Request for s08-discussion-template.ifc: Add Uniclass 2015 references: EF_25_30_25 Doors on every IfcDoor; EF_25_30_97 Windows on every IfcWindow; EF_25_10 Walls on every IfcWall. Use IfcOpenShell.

First a look at what the model holds.

```python
import ifcopenshell

model = ifcopenshell.open("s08-discussion-template.ifc")
print(model.schema)
print("classifications:", [c.Name for c in model.by_type("IfcClassification")])
for ifc_class in ("IfcDoor", "IfcRoof", "IfcStair", "IfcWall", "IfcWindow"):
    print(ifc_class, len(model.by_type(ifc_class)))
```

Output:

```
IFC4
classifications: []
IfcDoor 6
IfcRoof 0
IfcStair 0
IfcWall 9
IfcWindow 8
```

```python
import ifcopenshell
import ifcopenshell.api.classification

model = ifcopenshell.open("s08-discussion-template.ifc")

system = ifcopenshell.api.classification.add_classification(model, classification="Uniclass 2015")

codes = {
    "IfcDoor": ("EF_25_30_25", "Doors"),
    "IfcWindow": ("EF_25_30_97", "Windows"),
    "IfcWall": ("EF_25_10", "Walls"),
}
for ifc_class, (code, name) in codes.items():
    products = model.by_type(ifc_class)
    ifcopenshell.api.classification.add_reference(
        model, products=products, classification=system, identification=code, name=name
    )
    print(code, len(products))

model.write("s08-discussion-template_updated.ifc")
```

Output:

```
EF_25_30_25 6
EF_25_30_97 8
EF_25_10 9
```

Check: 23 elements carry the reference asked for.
